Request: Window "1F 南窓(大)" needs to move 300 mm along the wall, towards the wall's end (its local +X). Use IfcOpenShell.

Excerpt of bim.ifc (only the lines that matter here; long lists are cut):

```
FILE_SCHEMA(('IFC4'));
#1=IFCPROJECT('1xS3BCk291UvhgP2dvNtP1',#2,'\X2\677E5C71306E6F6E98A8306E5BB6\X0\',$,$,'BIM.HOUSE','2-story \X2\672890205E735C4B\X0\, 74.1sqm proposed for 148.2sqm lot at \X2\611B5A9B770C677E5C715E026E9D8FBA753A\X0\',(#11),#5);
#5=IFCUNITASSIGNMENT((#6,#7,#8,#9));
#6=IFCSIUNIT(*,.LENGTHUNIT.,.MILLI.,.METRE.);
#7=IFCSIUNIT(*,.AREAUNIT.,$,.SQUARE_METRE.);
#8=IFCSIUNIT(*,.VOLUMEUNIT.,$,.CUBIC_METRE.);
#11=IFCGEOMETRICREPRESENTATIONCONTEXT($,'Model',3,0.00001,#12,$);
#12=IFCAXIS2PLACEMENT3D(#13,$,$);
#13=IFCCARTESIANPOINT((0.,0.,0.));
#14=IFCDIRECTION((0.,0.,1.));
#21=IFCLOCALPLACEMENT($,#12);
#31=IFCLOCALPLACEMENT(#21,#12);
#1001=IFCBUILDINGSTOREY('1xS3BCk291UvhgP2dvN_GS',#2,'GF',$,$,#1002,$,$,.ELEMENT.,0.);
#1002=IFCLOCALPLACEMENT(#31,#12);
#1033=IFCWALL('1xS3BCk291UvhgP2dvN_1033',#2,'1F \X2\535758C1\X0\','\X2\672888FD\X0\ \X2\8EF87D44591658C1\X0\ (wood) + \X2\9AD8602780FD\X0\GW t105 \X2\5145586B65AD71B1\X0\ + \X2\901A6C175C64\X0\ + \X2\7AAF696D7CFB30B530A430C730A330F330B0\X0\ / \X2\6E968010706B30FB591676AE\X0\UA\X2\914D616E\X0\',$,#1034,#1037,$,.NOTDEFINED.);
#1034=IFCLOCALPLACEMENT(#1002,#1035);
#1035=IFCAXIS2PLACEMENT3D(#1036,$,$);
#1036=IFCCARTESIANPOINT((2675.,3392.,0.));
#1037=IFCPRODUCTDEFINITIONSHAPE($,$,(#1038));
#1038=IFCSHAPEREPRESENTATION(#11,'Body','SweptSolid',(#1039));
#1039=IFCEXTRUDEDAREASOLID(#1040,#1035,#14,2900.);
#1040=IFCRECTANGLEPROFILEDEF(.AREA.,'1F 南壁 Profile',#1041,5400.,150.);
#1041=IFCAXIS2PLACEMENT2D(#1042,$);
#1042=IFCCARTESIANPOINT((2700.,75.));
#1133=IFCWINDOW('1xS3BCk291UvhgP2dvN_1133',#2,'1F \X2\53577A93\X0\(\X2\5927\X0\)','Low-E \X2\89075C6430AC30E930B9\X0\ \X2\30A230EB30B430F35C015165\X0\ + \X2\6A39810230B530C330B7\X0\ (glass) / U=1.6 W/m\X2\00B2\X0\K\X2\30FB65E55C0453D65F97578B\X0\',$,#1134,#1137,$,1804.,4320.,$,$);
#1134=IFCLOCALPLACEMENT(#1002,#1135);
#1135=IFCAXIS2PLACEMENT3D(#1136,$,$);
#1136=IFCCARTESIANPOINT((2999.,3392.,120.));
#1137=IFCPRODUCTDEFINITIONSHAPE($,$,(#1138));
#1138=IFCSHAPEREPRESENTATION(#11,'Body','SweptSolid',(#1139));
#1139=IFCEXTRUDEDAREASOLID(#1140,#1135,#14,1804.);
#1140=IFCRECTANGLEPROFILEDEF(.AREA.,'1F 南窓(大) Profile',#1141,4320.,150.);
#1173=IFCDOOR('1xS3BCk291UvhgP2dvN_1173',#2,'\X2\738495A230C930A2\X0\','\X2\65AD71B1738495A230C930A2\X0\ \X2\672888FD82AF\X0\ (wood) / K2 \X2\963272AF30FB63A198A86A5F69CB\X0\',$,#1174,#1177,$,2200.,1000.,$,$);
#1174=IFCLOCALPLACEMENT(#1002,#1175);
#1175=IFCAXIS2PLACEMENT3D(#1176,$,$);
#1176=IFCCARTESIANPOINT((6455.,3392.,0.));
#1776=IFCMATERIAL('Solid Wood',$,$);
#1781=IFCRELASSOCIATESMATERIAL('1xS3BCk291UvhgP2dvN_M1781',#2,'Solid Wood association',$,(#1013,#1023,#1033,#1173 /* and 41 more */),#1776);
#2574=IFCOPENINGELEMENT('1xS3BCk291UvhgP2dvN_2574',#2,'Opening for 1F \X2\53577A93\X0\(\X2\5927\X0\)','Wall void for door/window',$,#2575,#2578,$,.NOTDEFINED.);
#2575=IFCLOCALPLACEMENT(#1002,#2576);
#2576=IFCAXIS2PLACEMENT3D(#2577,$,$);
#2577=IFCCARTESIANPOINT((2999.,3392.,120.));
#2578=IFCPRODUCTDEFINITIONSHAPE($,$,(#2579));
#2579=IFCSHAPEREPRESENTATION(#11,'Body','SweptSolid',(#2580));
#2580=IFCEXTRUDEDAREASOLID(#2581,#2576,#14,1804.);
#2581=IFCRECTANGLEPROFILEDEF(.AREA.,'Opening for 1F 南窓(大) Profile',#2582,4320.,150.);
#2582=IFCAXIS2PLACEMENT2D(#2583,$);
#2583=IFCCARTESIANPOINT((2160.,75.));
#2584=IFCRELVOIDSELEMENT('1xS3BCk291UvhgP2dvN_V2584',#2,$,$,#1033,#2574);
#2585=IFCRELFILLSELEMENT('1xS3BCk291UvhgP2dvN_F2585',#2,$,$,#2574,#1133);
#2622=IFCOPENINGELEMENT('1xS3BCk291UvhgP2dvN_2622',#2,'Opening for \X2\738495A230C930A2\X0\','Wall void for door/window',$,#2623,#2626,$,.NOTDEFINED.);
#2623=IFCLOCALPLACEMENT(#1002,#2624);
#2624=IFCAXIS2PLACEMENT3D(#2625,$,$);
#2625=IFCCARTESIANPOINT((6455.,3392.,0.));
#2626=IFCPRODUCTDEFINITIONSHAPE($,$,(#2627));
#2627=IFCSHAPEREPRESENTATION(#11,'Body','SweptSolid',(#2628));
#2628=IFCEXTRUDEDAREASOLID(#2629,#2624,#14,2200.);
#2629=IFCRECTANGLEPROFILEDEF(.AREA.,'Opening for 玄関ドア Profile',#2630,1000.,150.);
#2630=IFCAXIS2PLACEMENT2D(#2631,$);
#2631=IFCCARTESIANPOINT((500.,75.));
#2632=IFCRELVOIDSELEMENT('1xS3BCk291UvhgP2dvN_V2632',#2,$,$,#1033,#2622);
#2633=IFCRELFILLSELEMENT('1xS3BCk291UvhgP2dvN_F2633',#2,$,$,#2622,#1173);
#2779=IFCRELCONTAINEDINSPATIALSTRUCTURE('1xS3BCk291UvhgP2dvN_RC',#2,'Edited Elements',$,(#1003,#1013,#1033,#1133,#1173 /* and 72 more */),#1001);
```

```python
import ifcopenshell
import ifcopenshell.api.geometry
import ifcopenshell.util.placement

model = ifcopenshell.open("bim.ifc")

window = model.by_guid("1xS3BCk291UvhgP2dvN_1133")
opening = window.FillsVoids[0].RelatingOpeningElement
wall = opening.VoidsElements[0].RelatingBuildingElement

wall_matrix = ifcopenshell.util.placement.get_local_placement(wall.ObjectPlacement)
shift = wall_matrix[:3, 0] * 300.0
before = ifcopenshell.util.placement.get_local_placement(window.ObjectPlacement)[:3, 3].copy()

# The window is not placed relative to its opening, so move both.
for product in (opening, window):
    matrix = ifcopenshell.util.placement.get_local_placement(product.ObjectPlacement)
    matrix[:3, 3] += shift
    ifcopenshell.api.geometry.edit_object_placement(model, product=product, matrix=matrix, is_si=False)

after = ifcopenshell.util.placement.get_local_placement(window.ObjectPlacement)[:3, 3]
print("window moved by", (after - before).round(3) + 0.0)

model.write("bim_v2.ifc")
```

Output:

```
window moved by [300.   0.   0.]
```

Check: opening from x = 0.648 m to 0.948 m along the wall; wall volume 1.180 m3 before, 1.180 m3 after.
